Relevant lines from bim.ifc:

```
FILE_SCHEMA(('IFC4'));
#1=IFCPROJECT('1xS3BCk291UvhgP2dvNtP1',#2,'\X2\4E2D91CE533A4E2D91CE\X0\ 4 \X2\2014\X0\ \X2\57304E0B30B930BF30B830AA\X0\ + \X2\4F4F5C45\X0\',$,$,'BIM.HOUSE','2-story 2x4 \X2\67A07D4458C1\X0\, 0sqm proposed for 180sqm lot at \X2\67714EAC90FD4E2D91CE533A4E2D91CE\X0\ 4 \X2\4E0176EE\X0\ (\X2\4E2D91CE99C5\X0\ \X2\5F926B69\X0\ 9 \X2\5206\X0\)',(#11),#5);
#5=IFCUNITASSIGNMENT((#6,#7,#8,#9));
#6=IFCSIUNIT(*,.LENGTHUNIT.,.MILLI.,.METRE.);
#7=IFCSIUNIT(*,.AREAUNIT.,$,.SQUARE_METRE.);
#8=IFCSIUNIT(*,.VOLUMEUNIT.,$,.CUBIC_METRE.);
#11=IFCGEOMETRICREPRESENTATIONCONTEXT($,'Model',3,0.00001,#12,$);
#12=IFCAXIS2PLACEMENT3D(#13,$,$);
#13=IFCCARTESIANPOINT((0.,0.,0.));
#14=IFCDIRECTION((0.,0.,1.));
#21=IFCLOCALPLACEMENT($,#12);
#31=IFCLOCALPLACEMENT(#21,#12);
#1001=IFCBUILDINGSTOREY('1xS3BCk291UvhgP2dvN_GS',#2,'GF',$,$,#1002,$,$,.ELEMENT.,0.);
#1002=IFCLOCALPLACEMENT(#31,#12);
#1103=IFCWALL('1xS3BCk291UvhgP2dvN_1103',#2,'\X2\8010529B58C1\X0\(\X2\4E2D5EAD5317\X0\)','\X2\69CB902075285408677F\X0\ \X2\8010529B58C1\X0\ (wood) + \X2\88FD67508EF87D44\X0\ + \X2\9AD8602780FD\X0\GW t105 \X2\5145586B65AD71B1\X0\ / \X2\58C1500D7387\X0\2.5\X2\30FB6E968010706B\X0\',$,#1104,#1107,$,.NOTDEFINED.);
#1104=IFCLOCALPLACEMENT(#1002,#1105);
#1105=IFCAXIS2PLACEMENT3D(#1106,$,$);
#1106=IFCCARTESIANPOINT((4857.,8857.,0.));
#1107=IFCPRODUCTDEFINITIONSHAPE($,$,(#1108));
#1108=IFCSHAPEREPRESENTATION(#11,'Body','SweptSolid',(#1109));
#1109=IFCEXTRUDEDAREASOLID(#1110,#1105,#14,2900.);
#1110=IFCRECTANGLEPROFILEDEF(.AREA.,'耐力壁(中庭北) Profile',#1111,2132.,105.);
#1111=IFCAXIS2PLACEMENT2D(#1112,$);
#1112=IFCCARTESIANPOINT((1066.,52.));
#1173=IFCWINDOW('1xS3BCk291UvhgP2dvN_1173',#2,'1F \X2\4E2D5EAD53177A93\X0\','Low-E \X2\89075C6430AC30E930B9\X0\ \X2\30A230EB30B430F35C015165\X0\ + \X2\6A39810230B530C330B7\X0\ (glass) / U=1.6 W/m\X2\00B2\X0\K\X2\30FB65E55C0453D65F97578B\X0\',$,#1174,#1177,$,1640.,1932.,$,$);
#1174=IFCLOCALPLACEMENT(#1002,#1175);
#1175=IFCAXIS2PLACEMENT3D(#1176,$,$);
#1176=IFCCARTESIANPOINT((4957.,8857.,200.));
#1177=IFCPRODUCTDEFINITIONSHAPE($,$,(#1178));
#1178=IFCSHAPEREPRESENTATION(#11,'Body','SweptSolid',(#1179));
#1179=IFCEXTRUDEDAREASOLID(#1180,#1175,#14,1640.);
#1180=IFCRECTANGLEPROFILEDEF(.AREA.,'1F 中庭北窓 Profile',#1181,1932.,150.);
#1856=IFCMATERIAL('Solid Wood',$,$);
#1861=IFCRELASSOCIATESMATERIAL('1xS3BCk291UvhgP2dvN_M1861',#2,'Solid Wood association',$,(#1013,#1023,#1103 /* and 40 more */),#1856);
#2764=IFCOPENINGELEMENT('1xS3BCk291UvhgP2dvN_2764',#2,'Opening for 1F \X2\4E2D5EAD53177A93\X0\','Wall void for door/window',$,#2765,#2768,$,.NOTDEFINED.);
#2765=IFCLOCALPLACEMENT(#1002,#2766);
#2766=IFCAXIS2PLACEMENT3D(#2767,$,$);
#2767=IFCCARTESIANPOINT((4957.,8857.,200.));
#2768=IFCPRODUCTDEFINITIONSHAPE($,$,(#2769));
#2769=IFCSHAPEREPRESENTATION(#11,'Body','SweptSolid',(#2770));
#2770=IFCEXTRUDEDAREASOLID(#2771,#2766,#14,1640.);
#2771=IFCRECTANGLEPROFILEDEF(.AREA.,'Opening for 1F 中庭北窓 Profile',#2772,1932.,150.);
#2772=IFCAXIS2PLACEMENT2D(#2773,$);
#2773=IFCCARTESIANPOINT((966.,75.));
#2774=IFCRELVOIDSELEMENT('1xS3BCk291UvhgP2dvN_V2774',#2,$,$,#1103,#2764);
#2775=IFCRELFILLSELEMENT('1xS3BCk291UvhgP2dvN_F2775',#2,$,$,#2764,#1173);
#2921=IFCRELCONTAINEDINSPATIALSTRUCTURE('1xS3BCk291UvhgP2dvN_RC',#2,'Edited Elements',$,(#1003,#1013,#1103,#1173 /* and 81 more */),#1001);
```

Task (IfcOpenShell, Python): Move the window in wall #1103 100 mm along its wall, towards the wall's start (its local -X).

```python
import ifcopenshell
import ifcopenshell.api.geometry
import ifcopenshell.util.placement
import ifcopenshell.util.unit

model = ifcopenshell.open("bim.ifc")
unit_scale = ifcopenshell.util.unit.calculate_unit_scale(model)

window = model.by_id(1173)
opening = window.FillsVoids[0].RelatingOpeningElement
wall = opening.VoidsElements[0].RelatingBuildingElement

wall_matrix = ifcopenshell.util.placement.get_local_placement(wall.ObjectPlacement)
shift = wall_matrix[:3, 0] * -0.1 / unit_scale
before = ifcopenshell.util.placement.get_local_placement(window.ObjectPlacement)[:3, 3].copy()

# The window is not placed relative to its opening, so move both.
for product in (opening, window):
    matrix = ifcopenshell.util.placement.get_local_placement(product.ObjectPlacement)
    matrix[:3, 3] += shift
    ifcopenshell.api.geometry.edit_object_placement(model, product=product, matrix=matrix, is_si=False)

after = ifcopenshell.util.placement.get_local_placement(window.ObjectPlacement)[:3, 3]
print("window moved by", (after - before).round(3) + 0.0)

model.write("bim_updated.ifc")
```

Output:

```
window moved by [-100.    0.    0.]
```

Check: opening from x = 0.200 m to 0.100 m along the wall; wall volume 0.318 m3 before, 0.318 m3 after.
